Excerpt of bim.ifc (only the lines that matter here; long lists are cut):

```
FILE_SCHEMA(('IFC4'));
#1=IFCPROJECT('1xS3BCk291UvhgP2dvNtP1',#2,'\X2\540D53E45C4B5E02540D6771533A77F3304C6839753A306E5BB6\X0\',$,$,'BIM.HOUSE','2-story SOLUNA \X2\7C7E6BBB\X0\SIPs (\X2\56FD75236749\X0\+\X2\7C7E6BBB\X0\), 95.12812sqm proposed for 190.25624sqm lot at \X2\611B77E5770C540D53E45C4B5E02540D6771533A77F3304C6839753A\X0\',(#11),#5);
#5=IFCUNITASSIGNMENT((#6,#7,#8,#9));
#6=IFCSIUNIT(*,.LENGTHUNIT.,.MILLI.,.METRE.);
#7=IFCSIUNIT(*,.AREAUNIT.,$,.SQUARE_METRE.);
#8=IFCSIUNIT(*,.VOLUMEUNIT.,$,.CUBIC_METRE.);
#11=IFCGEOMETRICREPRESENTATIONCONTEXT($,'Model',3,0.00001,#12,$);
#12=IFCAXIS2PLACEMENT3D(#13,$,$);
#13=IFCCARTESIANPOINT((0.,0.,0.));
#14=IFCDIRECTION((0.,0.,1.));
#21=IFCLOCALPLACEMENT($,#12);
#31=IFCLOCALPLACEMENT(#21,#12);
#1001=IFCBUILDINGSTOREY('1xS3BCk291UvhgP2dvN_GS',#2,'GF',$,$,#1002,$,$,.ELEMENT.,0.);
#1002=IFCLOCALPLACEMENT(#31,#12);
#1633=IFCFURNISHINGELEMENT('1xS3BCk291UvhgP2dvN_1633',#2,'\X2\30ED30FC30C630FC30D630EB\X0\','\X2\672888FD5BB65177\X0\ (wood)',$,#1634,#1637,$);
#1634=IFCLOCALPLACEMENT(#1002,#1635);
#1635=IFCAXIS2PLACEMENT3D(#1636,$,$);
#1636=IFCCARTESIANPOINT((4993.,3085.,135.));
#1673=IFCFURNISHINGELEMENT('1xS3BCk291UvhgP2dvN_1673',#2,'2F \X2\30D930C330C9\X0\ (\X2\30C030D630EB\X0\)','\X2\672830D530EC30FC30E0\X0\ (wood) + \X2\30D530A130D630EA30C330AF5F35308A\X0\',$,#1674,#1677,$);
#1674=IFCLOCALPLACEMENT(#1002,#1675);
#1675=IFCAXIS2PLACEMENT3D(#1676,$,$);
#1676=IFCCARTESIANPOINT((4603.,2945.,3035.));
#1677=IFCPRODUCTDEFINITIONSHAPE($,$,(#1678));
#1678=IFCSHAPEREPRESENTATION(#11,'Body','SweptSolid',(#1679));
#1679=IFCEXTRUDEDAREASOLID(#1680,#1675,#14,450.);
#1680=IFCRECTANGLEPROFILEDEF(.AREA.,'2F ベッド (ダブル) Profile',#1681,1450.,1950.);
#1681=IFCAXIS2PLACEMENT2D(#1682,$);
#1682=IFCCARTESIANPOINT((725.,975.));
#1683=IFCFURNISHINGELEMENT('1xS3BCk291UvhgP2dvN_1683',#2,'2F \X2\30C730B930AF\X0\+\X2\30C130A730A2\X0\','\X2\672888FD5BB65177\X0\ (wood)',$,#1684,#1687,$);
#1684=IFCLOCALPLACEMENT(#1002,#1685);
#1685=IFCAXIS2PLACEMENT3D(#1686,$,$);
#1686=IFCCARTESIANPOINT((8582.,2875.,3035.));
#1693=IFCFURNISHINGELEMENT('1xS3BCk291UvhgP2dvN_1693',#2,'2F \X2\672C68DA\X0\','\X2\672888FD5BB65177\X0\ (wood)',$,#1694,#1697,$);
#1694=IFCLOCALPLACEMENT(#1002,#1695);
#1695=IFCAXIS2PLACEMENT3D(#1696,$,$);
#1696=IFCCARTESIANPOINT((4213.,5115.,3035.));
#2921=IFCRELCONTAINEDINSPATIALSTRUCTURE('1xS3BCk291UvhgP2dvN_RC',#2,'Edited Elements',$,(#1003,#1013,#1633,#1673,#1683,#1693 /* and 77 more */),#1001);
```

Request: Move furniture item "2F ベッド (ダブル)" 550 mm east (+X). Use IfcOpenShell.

```python
import ifcopenshell
import ifcopenshell.api.geometry
import ifcopenshell.util.placement
import ifcopenshell.util.unit

model = ifcopenshell.open("bim.ifc")
unit_scale = ifcopenshell.util.unit.calculate_unit_scale(model)

item = model.by_guid("1xS3BCk291UvhgP2dvN_1673")
matrix = ifcopenshell.util.placement.get_local_placement(item.ObjectPlacement)
matrix[0, 3] += 0.55 / unit_scale
ifcopenshell.api.geometry.edit_object_placement(model, product=item, matrix=matrix, is_si=False)

print(ifcopenshell.util.placement.get_local_placement(item.ObjectPlacement).round(3) + 0.0)

model.write("bim_updated.ifc")
```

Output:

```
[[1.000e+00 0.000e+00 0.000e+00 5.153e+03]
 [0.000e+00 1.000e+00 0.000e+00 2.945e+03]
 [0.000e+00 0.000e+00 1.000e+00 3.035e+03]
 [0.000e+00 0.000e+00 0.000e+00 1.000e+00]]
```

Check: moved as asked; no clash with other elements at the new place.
